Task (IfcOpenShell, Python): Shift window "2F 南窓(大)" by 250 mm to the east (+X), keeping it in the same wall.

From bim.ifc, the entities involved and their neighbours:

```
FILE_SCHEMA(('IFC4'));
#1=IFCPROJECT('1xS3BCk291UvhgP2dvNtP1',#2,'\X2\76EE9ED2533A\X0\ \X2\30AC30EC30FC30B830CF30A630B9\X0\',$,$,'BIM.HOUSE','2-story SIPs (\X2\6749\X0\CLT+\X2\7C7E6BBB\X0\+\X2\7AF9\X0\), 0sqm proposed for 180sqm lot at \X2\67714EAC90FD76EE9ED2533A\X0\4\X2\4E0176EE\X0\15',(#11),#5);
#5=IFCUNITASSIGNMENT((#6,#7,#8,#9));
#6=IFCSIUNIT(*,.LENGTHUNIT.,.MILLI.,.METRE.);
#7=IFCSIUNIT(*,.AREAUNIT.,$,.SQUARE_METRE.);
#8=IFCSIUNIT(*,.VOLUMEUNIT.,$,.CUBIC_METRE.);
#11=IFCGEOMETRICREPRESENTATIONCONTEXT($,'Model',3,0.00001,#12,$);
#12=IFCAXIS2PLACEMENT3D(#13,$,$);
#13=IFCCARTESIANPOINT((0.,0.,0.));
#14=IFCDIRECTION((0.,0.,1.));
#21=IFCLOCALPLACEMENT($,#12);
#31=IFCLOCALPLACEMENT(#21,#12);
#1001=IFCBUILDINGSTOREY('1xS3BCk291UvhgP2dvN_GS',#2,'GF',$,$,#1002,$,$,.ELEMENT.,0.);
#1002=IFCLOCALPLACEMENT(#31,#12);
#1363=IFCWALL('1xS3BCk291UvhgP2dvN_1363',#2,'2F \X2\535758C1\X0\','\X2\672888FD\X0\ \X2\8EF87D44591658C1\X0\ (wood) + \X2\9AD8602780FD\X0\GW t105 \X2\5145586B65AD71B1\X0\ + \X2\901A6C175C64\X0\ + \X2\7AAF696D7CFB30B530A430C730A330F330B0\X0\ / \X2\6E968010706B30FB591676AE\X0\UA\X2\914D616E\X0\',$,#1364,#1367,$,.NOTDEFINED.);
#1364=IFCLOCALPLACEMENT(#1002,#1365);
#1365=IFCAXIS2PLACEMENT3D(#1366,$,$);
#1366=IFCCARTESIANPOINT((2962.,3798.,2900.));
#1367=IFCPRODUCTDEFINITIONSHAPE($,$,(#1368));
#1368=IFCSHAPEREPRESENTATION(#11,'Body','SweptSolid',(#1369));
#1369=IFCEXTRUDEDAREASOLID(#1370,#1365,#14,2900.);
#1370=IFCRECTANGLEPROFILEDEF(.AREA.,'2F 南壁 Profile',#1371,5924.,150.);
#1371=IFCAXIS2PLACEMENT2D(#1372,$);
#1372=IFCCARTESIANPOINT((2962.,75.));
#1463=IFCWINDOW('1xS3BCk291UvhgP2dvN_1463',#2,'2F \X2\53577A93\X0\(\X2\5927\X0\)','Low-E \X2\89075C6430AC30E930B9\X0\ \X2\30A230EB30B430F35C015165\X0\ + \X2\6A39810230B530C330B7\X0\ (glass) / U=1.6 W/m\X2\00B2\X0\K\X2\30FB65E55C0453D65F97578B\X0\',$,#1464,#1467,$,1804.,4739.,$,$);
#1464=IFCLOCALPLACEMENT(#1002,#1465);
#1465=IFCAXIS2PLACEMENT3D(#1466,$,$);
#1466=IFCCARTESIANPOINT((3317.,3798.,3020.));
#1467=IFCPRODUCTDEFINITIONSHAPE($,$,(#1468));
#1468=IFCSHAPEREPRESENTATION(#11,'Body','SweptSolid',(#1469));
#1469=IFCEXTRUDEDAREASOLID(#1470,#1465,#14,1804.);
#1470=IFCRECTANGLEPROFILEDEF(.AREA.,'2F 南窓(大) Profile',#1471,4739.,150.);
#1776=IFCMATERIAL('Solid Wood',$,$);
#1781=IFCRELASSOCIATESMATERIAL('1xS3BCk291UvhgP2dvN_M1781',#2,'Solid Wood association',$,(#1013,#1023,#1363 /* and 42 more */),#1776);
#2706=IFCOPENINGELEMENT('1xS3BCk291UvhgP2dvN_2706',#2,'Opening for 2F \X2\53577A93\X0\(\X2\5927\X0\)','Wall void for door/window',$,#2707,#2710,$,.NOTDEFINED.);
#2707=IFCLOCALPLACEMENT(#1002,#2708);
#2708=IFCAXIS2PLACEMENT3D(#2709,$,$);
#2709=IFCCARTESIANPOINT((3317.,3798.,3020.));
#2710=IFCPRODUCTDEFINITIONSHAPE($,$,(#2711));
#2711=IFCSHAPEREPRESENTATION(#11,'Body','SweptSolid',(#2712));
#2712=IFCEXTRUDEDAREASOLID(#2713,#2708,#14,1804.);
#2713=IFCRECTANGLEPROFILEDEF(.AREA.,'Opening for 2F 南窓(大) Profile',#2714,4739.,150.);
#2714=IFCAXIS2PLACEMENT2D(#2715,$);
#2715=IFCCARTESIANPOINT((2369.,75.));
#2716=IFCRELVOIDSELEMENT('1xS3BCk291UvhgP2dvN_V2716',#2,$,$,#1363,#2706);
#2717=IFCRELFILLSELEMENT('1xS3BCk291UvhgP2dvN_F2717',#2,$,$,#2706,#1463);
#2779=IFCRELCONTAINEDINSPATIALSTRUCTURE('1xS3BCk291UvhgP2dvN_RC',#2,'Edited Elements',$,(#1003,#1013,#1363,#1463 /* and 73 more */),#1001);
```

```python
import ifcopenshell
import ifcopenshell.api.geometry
import ifcopenshell.util.placement
import ifcopenshell.util.unit

model = ifcopenshell.open("bim.ifc")
unit_scale = ifcopenshell.util.unit.calculate_unit_scale(model)

window = model.by_guid("1xS3BCk291UvhgP2dvN_1463")
opening = window.FillsVoids[0].RelatingOpeningElement
wall = opening.VoidsElements[0].RelatingBuildingElement

wall_matrix = ifcopenshell.util.placement.get_local_placement(wall.ObjectPlacement)
shift = wall_matrix[:3, 0] * 0.25 / unit_scale
before = ifcopenshell.util.placement.get_local_placement(window.ObjectPlacement)[:3, 3].copy()

# The window is not placed relative to its opening, so move both.
for product in (opening, window):
    matrix = ifcopenshell.util.placement.get_local_placement(product.ObjectPlacement)
    matrix[:3, 3] += shift
    ifcopenshell.api.geometry.edit_object_placement(model, product=product, matrix=matrix, is_si=False)

after = ifcopenshell.util.placement.get_local_placement(window.ObjectPlacement)[:3, 3]
print("window moved by", (after - before).round(3) + 0.0)

model.write("bim_rev.ifc")
```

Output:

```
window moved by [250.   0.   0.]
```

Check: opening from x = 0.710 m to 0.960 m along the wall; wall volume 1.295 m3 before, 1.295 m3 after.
